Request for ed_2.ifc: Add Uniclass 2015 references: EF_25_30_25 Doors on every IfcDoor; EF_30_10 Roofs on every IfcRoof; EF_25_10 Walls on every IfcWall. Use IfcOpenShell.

First a look at what the model holds.

```python
import ifcopenshell

model = ifcopenshell.open("ed_2.ifc")
print(model.schema)
print("classifications:", [c.Name for c in model.by_type("IfcClassification")])
for ifc_class in ("IfcDoor", "IfcRoof", "IfcStair", "IfcWall", "IfcWindow"):
    print(ifc_class, len(model.by_type(ifc_class)))
```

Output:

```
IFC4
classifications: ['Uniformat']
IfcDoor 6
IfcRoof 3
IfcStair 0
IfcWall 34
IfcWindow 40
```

```python
import ifcopenshell
import ifcopenshell.api.classification

model = ifcopenshell.open("ed_2.ifc")

system = ifcopenshell.api.classification.add_classification(model, classification="Uniclass 2015")

codes = {
    "IfcDoor": ("EF_25_30_25", "Doors"),
    "IfcRoof": ("EF_30_10", "Roofs"),
    "IfcWall": ("EF_25_10", "Walls"),
}
for ifc_class, (code, name) in codes.items():
    products = model.by_type(ifc_class)
    ifcopenshell.api.classification.add_reference(
        model, products=products, classification=system, identification=code, name=name
    )
    print(code, len(products))

model.write("ed_2_edited.ifc")
```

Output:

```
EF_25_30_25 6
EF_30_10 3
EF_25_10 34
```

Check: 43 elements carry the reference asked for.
